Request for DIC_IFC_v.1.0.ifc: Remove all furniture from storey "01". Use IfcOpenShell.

First a look at what the model holds.

```python
import ifcopenshell
import ifcopenshell.util.element

model = ifcopenshell.open("DIC_IFC_v.1.0.ifc")
print(model.schema)
storey = next(s for s in model.by_type("IfcBuildingStorey") if s.Name == "01")
furniture = [e for e in ifcopenshell.util.element.get_decomposition(storey) if e.is_a("IfcFurnishingElement")]
seen = {}
for e in furniture:
    element_type = ifcopenshell.util.element.get_type(e)
    name = element_type.Name if element_type not in (None, e) else None
    seen[name] = seen.get(name, 0) + 1
for name, count in sorted(seen.items(), key=str):
    print(count, "x", name)
```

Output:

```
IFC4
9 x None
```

```python
import ifcopenshell
import ifcopenshell.api.root
import ifcopenshell.util.element

model = ifcopenshell.open("DIC_IFC_v.1.0.ifc")

storey = next(s for s in model.by_type("IfcBuildingStorey") if s.Name == "01")
furniture = [e for e in ifcopenshell.util.element.get_decomposition(storey) if e.is_a("IfcFurnishingElement")]

for e in furniture:
    ifcopenshell.api.root.remove_product(model, product=e)
print(len(furniture), "removed")

model.write("DIC_IFC_v.1.0-out.ifc")
```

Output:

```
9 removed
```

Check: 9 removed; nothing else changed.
